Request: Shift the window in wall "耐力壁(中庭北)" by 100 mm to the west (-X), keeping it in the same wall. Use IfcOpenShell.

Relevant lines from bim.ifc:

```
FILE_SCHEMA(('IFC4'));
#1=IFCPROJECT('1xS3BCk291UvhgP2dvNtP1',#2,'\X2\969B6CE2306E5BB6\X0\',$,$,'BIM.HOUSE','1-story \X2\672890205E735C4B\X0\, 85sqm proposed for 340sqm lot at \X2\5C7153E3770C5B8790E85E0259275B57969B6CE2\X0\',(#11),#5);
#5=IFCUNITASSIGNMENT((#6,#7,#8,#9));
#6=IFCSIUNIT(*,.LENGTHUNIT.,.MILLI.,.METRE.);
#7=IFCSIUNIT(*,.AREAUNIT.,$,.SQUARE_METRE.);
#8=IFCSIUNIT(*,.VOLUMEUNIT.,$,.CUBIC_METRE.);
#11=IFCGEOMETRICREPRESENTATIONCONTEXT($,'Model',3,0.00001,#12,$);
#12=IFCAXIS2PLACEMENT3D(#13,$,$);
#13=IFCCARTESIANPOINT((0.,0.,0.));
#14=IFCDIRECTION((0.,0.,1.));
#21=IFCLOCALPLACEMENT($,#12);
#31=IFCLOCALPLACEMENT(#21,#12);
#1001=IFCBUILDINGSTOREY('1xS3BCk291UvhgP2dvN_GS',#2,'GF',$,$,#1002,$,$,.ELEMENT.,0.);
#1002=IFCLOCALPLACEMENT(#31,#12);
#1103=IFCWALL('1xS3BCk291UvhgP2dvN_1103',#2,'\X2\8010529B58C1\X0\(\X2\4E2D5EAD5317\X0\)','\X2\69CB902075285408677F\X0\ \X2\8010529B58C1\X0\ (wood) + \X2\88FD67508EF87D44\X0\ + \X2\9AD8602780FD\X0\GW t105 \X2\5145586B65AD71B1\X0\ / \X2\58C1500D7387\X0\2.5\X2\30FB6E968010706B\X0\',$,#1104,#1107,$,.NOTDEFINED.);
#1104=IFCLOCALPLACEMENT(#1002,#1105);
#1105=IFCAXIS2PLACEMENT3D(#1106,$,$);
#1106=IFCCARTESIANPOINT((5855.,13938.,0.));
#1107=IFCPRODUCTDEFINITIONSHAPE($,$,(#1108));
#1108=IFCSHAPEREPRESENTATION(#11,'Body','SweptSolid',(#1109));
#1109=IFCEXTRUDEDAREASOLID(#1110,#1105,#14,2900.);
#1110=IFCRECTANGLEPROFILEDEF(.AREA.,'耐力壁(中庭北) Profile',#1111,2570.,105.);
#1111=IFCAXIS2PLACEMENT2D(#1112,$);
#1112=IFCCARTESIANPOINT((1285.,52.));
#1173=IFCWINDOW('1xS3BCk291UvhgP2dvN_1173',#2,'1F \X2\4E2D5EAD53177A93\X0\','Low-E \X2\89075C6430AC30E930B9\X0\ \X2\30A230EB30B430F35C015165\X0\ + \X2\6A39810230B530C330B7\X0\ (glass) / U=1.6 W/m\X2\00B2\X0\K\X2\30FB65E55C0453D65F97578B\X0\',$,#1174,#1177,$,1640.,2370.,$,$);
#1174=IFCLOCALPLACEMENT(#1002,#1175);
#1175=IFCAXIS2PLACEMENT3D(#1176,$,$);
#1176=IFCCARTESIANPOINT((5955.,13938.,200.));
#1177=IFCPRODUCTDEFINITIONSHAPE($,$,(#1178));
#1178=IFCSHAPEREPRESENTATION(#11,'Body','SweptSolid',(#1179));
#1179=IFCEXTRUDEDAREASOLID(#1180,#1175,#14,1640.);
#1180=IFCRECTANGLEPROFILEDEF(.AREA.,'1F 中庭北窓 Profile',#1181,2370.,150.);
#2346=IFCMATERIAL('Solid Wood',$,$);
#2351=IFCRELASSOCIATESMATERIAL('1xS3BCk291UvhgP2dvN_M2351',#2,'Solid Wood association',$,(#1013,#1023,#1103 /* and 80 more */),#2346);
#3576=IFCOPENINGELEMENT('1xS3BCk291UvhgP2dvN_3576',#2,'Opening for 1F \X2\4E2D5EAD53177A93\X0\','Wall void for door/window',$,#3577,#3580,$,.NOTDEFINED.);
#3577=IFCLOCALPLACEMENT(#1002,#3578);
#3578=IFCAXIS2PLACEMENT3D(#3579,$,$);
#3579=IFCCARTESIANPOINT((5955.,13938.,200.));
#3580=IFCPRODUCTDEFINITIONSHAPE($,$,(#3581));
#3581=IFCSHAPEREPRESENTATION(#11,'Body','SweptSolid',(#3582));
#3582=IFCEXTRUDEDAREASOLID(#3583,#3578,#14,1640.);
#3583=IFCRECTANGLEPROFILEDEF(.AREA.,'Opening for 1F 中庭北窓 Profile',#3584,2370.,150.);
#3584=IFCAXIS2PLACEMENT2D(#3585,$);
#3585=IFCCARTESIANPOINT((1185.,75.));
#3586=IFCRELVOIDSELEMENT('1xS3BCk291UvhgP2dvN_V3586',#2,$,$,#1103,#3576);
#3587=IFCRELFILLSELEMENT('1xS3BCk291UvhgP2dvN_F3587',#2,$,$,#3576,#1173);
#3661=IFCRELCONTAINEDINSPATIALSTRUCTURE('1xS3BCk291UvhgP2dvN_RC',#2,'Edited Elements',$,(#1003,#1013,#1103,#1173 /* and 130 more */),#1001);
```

```python
import ifcopenshell
import ifcopenshell.api.geometry
import ifcopenshell.util.placement

model = ifcopenshell.open("bim.ifc")

window = model.by_guid("1xS3BCk291UvhgP2dvN_1173")
opening = window.FillsVoids[0].RelatingOpeningElement
wall = opening.VoidsElements[0].RelatingBuildingElement

wall_matrix = ifcopenshell.util.placement.get_local_placement(wall.ObjectPlacement)
shift = wall_matrix[:3, 0] * -100.0
before = ifcopenshell.util.placement.get_local_placement(window.ObjectPlacement)[:3, 3].copy()

# The window is not placed relative to its opening, so move both.
for product in (opening, window):
    matrix = ifcopenshell.util.placement.get_local_placement(product.ObjectPlacement)
    matrix[:3, 3] += shift
    ifcopenshell.api.geometry.edit_object_placement(model, product=product, matrix=matrix, is_si=False)

after = ifcopenshell.util.placement.get_local_placement(window.ObjectPlacement)[:3, 3]
print("window moved by", (after - before).round(3) + 0.0)

model.write("bim_edited.ifc")
```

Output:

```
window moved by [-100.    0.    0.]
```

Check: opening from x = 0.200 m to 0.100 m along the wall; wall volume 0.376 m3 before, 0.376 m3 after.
